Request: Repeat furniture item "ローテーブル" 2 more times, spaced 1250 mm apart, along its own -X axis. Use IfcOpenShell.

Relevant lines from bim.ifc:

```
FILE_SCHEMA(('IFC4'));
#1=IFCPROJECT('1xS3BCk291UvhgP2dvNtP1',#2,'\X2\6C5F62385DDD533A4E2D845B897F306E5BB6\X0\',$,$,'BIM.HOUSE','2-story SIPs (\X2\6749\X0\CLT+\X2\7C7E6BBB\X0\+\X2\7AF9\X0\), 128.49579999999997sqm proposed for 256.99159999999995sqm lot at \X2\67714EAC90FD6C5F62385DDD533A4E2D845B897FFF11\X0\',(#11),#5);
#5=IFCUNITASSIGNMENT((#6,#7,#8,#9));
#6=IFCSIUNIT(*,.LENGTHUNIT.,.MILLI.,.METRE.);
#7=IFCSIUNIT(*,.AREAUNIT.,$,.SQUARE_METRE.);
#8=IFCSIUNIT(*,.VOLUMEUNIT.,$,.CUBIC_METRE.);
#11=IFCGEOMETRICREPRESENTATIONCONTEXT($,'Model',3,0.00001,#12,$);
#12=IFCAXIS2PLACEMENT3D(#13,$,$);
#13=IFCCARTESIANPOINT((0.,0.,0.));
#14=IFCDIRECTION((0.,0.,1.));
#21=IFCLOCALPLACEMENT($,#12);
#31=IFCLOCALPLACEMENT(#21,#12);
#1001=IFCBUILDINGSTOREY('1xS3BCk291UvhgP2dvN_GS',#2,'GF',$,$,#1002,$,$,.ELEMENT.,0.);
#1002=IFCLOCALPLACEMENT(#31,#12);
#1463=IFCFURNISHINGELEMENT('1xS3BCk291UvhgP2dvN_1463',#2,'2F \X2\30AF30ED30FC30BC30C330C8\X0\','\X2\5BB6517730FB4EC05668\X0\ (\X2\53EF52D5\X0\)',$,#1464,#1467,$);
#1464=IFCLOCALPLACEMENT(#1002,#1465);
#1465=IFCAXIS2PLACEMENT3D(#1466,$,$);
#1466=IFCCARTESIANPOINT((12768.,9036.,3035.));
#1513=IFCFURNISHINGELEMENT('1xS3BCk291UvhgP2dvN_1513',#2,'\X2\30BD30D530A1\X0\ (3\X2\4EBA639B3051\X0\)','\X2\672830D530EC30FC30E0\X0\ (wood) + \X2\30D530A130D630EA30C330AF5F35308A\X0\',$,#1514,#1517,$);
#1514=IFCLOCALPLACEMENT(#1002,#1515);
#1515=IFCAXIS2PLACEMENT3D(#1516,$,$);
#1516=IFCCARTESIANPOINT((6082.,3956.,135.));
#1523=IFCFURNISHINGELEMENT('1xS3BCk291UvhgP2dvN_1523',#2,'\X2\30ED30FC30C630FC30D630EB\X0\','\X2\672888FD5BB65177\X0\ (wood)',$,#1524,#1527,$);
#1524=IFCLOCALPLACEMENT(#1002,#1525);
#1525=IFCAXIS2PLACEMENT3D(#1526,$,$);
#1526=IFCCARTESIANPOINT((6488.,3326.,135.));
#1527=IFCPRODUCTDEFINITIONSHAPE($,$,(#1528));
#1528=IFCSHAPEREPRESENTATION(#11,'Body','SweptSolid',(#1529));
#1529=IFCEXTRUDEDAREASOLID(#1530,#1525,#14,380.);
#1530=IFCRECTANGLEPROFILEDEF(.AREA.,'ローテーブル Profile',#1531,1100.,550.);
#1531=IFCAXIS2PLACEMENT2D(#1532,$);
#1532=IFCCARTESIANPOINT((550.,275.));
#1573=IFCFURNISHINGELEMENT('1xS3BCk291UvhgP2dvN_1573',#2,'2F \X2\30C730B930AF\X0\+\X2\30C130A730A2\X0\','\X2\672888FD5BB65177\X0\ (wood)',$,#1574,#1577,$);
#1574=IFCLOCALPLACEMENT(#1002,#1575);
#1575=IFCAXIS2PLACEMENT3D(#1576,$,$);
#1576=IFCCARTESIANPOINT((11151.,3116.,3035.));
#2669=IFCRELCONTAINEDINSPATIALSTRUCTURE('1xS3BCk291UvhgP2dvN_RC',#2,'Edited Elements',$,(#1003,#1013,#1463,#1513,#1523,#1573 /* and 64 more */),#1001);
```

```python
import ifcopenshell
import ifcopenshell.api.geometry
import ifcopenshell.api.root
import ifcopenshell.util.element
import ifcopenshell.util.placement

model = ifcopenshell.open("bim.ifc")


def reuse_history(source, copy):
    """copy_class also copies each property set's owner history, people and application; keep the originals."""
    for rel in copy.IsDefinedBy:
        if rel.is_a("IfcRelDefinesByProperties") and (history := rel.RelatingPropertyDefinition.OwnerHistory):
            rel.RelatingPropertyDefinition.OwnerHistory = source.OwnerHistory
            ifcopenshell.util.element.remove_deep2(model, history)


source = model.by_guid("1xS3BCk291UvhgP2dvN_1523")
base = ifcopenshell.util.placement.get_local_placement(source.ObjectPlacement)
step = -base[:3, 0] * 1250.0

for i in range(1, 3):
    copy = ifcopenshell.api.root.copy_class(model, product=source)
    copy.Representation = ifcopenshell.util.element.copy_deep(
        model, source.Representation, exclude=["IfcGeometricRepresentationContext", "IfcRepresentationMap"]
    )
    reuse_history(source, copy)
    matrix = base.copy()
    matrix[:3, 3] += i * step
    print("added at", matrix[:3, 3].round(3) + 0.0)
    ifcopenshell.api.geometry.edit_object_placement(model, product=copy, matrix=matrix, is_si=False)

model.write("bim_v2.ifc")
```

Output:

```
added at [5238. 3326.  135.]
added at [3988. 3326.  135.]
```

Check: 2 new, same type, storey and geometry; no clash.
